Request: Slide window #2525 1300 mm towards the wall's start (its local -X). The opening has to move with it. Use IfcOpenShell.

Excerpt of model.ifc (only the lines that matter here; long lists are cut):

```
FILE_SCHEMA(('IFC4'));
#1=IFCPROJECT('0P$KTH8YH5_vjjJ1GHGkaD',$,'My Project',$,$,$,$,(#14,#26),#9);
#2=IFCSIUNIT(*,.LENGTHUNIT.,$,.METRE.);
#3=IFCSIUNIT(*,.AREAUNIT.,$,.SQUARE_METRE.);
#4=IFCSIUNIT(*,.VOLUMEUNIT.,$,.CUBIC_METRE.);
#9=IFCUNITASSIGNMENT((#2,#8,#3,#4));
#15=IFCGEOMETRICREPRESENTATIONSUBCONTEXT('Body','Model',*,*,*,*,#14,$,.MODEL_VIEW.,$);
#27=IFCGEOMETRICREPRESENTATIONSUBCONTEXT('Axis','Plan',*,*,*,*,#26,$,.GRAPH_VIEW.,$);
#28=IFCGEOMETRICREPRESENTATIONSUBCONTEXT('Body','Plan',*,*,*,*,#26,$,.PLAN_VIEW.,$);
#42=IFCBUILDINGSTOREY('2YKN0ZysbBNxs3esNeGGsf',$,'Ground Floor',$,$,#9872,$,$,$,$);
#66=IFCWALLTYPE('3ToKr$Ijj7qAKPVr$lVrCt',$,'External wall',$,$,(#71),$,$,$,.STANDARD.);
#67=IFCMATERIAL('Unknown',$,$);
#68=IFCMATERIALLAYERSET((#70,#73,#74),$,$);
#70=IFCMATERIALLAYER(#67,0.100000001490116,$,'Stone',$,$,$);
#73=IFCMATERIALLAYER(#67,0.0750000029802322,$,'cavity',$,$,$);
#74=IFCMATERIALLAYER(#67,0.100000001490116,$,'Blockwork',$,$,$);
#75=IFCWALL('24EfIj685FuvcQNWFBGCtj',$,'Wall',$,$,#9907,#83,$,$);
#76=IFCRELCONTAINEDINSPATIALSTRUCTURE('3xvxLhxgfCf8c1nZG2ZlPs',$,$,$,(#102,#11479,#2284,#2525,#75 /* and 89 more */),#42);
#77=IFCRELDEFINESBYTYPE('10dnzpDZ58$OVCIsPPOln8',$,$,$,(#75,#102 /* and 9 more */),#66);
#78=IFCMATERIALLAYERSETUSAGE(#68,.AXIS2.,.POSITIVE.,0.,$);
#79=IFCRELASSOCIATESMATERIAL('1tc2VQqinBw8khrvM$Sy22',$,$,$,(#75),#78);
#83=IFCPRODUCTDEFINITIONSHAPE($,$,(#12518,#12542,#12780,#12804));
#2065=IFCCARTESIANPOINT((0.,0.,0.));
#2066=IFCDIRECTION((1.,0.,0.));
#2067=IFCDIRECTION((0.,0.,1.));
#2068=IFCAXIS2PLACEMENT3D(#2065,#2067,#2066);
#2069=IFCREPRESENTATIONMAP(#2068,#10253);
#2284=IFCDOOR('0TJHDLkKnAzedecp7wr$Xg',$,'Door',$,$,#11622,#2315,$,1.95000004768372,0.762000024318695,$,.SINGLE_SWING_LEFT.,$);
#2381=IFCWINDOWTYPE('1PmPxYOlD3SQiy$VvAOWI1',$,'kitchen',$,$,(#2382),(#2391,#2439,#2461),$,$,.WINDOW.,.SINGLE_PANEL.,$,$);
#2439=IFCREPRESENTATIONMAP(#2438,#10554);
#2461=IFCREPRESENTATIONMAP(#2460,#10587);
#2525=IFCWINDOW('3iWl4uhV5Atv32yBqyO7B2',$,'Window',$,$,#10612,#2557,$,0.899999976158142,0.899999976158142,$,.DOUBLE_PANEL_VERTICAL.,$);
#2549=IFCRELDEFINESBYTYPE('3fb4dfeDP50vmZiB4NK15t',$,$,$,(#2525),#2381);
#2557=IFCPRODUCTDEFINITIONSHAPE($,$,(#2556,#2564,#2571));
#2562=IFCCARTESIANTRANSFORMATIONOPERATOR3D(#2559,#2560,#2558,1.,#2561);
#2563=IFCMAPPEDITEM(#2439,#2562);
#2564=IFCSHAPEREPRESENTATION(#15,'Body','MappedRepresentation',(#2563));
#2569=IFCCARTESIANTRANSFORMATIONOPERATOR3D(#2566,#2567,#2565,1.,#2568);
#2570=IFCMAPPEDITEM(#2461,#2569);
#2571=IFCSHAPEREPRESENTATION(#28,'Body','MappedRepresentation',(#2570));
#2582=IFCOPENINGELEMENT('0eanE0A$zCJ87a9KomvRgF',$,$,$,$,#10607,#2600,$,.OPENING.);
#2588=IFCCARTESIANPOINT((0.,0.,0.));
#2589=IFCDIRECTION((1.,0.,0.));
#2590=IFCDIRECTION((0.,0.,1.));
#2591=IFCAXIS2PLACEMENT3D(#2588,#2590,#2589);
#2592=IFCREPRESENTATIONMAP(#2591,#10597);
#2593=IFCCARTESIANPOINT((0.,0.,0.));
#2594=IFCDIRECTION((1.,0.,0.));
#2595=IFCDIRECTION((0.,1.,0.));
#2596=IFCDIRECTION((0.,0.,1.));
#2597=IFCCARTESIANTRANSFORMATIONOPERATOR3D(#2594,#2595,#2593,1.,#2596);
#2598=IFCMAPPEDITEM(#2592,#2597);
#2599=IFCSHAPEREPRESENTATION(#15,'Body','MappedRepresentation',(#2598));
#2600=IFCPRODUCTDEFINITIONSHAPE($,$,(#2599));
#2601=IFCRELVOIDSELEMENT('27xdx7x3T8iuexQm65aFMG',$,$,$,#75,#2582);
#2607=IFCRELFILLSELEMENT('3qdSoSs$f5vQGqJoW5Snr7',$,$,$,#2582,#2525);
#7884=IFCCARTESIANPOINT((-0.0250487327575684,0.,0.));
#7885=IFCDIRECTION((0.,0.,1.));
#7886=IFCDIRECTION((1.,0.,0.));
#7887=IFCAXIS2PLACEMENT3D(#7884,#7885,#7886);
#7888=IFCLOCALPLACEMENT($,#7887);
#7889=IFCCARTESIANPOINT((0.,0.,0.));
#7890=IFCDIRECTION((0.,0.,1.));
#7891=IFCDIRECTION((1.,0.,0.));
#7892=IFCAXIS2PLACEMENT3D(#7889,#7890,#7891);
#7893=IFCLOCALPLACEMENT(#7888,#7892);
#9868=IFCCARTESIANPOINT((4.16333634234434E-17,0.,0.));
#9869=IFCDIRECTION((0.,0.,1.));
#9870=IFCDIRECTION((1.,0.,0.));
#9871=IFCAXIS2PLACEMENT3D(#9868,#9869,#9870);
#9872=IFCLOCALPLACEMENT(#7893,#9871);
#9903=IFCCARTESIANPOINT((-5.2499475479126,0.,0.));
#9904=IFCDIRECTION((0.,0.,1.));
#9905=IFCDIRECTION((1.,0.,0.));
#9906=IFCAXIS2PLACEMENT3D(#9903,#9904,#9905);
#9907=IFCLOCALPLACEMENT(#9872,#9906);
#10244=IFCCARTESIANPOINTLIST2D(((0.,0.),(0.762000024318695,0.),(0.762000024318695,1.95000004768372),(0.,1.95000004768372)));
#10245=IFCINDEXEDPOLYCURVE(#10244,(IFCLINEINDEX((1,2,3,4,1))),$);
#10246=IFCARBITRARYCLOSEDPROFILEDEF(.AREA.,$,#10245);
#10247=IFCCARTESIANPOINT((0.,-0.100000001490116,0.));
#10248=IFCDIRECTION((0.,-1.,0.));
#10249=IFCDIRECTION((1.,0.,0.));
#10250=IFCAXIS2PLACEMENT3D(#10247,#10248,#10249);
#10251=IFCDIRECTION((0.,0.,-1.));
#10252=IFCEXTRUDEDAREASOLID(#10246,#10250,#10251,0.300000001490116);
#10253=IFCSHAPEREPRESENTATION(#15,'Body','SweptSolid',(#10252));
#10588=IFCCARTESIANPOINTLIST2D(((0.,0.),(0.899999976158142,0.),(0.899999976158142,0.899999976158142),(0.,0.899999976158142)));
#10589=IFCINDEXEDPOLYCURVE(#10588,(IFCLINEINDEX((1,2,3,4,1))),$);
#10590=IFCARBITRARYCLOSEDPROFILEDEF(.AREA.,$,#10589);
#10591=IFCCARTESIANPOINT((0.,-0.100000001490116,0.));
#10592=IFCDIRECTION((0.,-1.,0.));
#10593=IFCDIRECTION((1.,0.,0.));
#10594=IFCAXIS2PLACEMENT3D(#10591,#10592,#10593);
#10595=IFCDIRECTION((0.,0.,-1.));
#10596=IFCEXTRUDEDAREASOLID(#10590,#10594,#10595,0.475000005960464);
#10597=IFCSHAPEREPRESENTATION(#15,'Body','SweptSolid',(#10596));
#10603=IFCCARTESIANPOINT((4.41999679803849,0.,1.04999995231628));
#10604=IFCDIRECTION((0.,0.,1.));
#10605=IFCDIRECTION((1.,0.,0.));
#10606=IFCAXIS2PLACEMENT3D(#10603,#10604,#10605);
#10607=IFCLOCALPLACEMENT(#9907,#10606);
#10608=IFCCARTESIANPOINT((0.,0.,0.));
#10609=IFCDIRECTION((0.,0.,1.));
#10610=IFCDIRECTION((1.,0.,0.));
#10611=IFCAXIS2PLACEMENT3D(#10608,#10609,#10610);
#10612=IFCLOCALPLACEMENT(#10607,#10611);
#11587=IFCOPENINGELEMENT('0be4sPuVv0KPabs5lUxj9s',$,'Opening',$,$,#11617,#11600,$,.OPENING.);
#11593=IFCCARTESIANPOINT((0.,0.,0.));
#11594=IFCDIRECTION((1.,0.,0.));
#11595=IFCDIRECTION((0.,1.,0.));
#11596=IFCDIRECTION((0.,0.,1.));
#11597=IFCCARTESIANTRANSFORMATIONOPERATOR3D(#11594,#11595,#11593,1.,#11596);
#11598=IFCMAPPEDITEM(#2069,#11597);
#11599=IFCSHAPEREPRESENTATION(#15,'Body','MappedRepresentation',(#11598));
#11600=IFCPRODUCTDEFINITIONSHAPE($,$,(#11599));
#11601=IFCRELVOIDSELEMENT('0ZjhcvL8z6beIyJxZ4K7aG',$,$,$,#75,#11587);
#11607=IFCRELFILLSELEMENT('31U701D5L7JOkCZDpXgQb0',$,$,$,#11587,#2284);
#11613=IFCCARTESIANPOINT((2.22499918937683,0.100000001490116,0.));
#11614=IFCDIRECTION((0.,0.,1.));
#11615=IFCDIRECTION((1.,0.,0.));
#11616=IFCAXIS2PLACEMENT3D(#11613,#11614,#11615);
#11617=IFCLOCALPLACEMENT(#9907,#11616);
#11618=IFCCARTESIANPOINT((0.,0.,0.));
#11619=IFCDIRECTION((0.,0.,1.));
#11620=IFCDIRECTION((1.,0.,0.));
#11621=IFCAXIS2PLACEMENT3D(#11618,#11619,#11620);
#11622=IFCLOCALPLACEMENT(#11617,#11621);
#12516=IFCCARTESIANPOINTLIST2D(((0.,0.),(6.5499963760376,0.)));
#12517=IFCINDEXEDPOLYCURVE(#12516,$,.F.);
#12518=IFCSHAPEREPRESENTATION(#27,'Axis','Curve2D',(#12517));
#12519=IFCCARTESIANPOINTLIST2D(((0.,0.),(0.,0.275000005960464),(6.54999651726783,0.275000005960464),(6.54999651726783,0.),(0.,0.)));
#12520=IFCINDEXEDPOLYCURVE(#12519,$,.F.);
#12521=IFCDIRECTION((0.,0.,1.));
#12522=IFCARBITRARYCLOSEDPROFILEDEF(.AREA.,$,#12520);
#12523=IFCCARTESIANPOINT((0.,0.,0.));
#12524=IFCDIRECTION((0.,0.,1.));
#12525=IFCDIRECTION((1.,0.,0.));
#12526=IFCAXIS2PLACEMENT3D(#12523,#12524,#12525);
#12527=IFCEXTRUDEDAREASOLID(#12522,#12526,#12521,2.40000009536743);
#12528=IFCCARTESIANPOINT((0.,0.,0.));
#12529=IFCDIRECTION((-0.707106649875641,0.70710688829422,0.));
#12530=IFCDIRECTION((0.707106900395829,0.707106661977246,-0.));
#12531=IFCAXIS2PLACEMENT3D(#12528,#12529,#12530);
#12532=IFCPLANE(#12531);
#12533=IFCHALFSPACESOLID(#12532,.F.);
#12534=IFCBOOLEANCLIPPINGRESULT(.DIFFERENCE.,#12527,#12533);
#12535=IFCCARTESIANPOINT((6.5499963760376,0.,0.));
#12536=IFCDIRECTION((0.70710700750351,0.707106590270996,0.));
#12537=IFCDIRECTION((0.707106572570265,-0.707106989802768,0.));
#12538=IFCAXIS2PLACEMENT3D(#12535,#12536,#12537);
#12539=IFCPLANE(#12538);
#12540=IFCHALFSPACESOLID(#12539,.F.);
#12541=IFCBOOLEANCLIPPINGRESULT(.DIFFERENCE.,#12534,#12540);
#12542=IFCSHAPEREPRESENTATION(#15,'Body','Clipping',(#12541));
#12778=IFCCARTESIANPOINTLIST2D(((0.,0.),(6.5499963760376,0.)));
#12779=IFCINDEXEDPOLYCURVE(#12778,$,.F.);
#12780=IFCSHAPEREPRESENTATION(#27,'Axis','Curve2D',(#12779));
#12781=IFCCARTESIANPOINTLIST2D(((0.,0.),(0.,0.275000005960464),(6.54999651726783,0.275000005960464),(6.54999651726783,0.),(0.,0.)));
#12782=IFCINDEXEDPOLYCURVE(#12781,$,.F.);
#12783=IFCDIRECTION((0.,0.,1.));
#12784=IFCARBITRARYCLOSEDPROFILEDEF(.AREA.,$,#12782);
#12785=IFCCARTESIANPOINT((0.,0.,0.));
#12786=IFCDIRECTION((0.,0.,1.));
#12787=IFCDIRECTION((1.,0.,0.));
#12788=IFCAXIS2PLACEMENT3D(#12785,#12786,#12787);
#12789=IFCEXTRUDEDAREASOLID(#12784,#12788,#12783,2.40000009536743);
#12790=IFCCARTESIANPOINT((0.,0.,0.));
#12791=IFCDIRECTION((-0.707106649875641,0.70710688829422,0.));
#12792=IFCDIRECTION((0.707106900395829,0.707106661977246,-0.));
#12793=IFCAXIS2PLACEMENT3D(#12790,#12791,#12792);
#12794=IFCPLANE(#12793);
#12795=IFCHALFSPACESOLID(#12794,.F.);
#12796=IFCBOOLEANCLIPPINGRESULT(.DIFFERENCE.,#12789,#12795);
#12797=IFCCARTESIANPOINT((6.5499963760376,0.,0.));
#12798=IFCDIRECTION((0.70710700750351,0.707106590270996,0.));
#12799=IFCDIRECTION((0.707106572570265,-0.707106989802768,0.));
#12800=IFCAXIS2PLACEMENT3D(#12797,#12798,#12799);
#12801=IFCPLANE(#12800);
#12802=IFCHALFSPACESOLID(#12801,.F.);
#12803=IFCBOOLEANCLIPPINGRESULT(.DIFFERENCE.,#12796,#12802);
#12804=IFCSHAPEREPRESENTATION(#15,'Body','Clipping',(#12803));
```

```python
import ifcopenshell
import ifcopenshell.api.geometry
import ifcopenshell.util.placement

model = ifcopenshell.open("model.ifc")

window = model.by_guid("3iWl4uhV5Atv32yBqyO7B2")
opening = window.FillsVoids[0].RelatingOpeningElement
wall = opening.VoidsElements[0].RelatingBuildingElement

wall_matrix = ifcopenshell.util.placement.get_local_placement(wall.ObjectPlacement)
shift = wall_matrix[:3, 0] * -1.3
before = ifcopenshell.util.placement.get_local_placement(window.ObjectPlacement)[:3, 3].copy()

# The window is placed relative to its opening, so it follows when the opening moves.
matrix = ifcopenshell.util.placement.get_local_placement(opening.ObjectPlacement)
matrix[:3, 3] += shift
ifcopenshell.api.geometry.edit_object_placement(
    model, product=opening, matrix=matrix, is_si=False, should_transform_children=True
)

after = ifcopenshell.util.placement.get_local_placement(window.ObjectPlacement)[:3, 3]
print("window moved by", (after - before).round(3) + 0.0)

model.write("model_v2.ifc")
```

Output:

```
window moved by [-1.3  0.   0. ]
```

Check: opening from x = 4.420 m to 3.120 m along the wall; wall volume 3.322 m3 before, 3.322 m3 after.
